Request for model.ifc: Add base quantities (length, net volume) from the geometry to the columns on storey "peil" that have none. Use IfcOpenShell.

First a look at what the model holds.

```python
import ifcopenshell
import ifcopenshell.util.element
import ifcopenshell.util.unit

model = ifcopenshell.open("model.ifc")
print(model.schema)
for unit_type in ("LENGTHUNIT", "AREAUNIT", "VOLUMEUNIT"):
    print(unit_type, ifcopenshell.util.unit.calculate_unit_scale(model, unit_type))
storey = next(s for s in model.by_type("IfcBuildingStorey") if s.Name == "peil")
columns = [e for e in ifcopenshell.util.element.get_decomposition(storey) if e.is_a("IfcColumn")]
for e in sorted(columns, key=lambda e: e.id()):
    print(e.id(), e.is_a(), e.Name, list(ifcopenshell.util.element.get_psets(e, qtos_only=True)), sep=" | ")
```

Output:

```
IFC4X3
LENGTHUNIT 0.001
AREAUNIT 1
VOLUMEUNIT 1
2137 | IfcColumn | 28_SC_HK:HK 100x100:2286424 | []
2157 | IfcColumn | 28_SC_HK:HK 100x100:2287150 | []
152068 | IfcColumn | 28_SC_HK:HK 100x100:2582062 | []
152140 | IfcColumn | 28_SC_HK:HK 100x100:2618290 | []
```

```python
import ifcopenshell
import ifcopenshell.api.pset
import ifcopenshell.geom
import ifcopenshell.util.element
import ifcopenshell.util.shape
import ifcopenshell.util.unit

model = ifcopenshell.open("model.ifc")
unit_scale = ifcopenshell.util.unit.calculate_unit_scale(model)
volume_scale = ifcopenshell.util.unit.calculate_unit_scale(model, "VOLUMEUNIT")
settings = ifcopenshell.geom.settings()

storey = next(s for s in model.by_type("IfcBuildingStorey") if s.Name == "peil")
columns = [e for e in ifcopenshell.util.element.get_decomposition(storey) if e.is_a("IfcColumn")]

for e in sorted(columns, key=lambda e: e.id()):
    if ifcopenshell.util.element.get_psets(e, qtos_only=True, should_inherit=False):
        continue
    # Geometry comes back in metres, in the element's own axes.
    shape = ifcopenshell.geom.create_shape(settings, e)
    values = {
        "Length": ifcopenshell.util.shape.get_z(shape.geometry) / unit_scale,
        "NetVolume": ifcopenshell.util.shape.get_volume(shape.geometry) / volume_scale,
    }
    qto = ifcopenshell.api.pset.add_qto(model, product=e, name="Qto_ColumnBaseQuantities")
    ifcopenshell.api.pset.edit_qto(model, qto=qto, properties=values)
    print(e.id(), {k: round(v, 3) for k, v in values.items()})

model.write("model-out.ifc")
```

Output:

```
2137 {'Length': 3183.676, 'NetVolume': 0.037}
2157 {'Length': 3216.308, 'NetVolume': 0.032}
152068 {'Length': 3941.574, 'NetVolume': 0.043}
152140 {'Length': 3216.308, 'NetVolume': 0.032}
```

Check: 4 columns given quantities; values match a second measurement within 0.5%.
